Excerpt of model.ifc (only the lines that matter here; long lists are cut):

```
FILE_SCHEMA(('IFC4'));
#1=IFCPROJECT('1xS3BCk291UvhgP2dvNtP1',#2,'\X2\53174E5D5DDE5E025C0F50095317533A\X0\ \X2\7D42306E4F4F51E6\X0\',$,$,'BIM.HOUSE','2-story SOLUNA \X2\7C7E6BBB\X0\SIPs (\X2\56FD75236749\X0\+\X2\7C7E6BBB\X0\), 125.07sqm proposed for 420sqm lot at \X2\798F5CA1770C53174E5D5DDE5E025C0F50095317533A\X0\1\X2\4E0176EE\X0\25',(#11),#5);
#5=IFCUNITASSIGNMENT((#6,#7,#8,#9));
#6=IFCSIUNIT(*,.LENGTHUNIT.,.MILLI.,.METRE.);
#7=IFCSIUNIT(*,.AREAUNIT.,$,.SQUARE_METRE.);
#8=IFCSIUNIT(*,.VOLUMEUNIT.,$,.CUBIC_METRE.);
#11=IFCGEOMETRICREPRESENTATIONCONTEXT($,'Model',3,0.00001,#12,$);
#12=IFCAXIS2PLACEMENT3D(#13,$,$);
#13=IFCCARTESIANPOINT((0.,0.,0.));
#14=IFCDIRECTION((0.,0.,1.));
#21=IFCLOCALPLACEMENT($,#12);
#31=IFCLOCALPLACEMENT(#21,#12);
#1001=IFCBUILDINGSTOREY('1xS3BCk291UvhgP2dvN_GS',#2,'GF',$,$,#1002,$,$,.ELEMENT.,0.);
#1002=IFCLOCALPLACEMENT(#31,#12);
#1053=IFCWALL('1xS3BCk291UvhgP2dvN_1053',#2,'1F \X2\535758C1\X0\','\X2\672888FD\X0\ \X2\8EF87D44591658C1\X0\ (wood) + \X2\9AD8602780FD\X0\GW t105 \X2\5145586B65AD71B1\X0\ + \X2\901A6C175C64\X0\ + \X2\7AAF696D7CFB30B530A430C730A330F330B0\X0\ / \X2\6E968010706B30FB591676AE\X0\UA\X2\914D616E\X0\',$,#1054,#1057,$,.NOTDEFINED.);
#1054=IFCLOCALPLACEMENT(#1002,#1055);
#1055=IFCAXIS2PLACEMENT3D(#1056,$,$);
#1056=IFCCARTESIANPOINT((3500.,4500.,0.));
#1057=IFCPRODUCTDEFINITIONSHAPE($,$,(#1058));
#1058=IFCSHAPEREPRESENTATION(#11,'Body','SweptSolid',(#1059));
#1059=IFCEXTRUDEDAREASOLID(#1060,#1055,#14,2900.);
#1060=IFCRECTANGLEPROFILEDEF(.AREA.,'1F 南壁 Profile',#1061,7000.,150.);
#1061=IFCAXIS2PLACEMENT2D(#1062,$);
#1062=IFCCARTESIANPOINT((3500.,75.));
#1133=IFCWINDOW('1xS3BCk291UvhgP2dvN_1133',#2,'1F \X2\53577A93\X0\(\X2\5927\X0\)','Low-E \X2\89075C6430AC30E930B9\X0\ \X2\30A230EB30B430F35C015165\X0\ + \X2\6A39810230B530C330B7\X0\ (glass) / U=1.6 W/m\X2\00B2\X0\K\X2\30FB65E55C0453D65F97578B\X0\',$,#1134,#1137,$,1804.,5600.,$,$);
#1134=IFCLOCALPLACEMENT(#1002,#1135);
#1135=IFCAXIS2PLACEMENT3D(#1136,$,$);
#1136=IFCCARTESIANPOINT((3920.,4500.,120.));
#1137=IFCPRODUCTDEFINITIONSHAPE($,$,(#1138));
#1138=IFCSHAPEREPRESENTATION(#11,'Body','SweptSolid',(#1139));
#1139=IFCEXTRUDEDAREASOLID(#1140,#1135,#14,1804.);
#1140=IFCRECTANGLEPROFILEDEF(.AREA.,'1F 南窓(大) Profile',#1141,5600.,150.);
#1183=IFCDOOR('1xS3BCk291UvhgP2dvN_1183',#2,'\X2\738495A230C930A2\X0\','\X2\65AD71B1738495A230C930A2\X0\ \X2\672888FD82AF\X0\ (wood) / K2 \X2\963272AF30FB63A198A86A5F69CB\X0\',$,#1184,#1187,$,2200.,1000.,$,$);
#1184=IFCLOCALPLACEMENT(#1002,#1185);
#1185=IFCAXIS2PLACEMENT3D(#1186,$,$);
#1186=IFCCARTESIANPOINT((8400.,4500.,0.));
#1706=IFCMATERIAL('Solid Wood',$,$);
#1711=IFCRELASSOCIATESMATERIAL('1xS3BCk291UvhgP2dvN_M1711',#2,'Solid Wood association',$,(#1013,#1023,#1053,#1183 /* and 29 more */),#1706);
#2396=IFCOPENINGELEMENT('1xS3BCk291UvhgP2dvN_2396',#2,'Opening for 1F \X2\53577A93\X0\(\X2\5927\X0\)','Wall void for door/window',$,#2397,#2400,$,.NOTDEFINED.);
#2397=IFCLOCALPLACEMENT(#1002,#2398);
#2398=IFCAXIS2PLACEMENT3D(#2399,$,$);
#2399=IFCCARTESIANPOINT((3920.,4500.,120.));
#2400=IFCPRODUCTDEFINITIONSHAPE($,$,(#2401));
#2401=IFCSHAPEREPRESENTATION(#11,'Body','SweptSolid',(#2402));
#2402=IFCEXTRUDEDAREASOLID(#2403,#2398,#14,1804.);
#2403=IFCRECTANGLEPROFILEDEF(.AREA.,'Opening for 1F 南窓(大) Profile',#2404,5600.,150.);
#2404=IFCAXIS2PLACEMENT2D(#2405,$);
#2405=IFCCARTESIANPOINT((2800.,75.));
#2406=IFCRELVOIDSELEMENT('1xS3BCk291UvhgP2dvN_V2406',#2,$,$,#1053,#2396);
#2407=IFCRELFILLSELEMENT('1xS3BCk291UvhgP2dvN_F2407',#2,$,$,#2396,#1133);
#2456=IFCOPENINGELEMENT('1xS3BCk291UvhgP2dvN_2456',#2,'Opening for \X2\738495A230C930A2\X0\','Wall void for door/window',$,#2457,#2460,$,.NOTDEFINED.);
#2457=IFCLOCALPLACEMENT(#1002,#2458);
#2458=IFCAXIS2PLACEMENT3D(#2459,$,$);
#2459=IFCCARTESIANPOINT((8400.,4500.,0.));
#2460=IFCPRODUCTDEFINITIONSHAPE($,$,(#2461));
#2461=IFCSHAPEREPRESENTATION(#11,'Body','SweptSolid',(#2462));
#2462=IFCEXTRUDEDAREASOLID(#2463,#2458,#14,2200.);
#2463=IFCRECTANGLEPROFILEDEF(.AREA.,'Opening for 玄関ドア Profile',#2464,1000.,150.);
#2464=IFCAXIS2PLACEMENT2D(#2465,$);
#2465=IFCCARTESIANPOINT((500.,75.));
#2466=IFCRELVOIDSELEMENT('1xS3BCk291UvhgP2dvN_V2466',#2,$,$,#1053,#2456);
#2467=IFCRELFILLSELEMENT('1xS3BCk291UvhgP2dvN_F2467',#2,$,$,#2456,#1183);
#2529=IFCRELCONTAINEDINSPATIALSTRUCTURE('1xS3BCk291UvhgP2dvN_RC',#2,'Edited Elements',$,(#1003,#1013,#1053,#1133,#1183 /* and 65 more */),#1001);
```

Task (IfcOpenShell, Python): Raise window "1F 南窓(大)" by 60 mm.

```python
import numpy as np
import ifcopenshell
import ifcopenshell.api.geometry
import ifcopenshell.util.placement
import ifcopenshell.util.unit

model = ifcopenshell.open("model.ifc")
unit_scale = ifcopenshell.util.unit.calculate_unit_scale(model)

window = model.by_guid("1xS3BCk291UvhgP2dvN_1133")
opening = window.FillsVoids[0].RelatingOpeningElement
dz = 0.06 / unit_scale

shift = np.array([0.0, 0.0, dz])
# The window is not placed relative to its opening, so move both.
for product in (opening, window):
    matrix = ifcopenshell.util.placement.get_local_placement(product.ObjectPlacement)
    matrix[:3, 3] += shift
    ifcopenshell.api.geometry.edit_object_placement(model, product=product, matrix=matrix, is_si=False)

print(f"moved by {dz * unit_scale:+.3f} m")

model.write("model_rev.ifc")
```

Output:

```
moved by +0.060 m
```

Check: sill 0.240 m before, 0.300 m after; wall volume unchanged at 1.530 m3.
